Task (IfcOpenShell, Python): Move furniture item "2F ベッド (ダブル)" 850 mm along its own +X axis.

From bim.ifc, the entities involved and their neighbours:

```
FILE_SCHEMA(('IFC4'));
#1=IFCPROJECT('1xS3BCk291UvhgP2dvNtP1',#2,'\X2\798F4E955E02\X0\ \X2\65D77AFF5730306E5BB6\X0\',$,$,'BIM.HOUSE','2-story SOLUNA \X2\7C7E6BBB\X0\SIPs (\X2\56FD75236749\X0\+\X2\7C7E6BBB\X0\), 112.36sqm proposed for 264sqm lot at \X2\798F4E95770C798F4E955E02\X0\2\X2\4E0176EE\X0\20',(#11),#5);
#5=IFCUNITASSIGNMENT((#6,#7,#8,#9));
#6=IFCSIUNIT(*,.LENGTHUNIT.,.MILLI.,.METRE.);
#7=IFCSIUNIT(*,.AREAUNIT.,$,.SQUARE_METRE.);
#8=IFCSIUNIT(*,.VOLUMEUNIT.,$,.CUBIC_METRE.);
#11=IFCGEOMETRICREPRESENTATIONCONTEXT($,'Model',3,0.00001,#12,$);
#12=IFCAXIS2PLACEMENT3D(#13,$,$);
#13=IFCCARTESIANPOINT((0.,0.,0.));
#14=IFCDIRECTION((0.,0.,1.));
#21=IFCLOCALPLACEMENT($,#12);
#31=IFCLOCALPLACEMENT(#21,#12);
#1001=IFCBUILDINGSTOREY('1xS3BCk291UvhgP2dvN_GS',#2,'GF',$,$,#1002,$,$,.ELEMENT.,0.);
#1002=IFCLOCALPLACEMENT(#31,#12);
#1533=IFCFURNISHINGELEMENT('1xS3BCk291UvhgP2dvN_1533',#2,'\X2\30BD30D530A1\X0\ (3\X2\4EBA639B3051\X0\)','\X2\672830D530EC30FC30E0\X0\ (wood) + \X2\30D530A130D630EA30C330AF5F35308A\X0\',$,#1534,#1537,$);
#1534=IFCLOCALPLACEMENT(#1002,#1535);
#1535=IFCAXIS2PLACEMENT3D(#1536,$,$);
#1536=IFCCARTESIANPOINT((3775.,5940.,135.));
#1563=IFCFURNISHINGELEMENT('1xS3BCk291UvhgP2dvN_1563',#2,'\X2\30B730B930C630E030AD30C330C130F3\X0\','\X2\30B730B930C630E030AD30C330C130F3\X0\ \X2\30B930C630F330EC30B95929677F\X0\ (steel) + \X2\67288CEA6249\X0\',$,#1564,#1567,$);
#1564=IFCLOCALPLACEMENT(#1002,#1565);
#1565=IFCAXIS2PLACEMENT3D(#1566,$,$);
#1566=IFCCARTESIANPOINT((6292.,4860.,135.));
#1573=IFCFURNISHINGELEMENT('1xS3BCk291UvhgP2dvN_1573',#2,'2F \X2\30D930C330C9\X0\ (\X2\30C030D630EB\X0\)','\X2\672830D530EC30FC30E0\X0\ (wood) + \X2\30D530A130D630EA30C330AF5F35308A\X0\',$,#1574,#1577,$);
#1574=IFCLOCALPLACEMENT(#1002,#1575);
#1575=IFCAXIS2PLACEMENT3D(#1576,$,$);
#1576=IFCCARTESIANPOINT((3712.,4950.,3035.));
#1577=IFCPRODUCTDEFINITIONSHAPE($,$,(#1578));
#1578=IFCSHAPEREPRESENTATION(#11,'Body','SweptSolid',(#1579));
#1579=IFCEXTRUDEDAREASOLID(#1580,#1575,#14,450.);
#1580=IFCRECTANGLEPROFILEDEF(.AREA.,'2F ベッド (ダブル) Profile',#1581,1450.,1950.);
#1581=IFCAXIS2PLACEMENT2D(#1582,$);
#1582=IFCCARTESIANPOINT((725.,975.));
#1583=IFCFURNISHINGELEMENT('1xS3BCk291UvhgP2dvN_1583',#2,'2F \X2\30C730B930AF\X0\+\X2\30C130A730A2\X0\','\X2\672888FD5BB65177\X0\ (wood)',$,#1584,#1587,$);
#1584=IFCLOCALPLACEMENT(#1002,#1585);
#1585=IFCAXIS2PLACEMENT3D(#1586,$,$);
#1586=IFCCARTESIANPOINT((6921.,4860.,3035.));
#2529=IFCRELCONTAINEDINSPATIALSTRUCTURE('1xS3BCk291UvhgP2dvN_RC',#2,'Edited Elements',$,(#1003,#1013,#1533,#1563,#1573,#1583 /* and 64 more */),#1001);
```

```python
import ifcopenshell
import ifcopenshell.api.geometry
import ifcopenshell.util.placement
import ifcopenshell.util.unit

model = ifcopenshell.open("bim.ifc")
unit_scale = ifcopenshell.util.unit.calculate_unit_scale(model)

item = model.by_id(1573)
matrix = ifcopenshell.util.placement.get_local_placement(item.ObjectPlacement)
matrix[:3, 3] += matrix[:3, 0] * 0.85 / unit_scale
ifcopenshell.api.geometry.edit_object_placement(model, product=item, matrix=matrix, is_si=False)

print(ifcopenshell.util.placement.get_local_placement(item.ObjectPlacement).round(3) + 0.0)

model.write("bim_v2.ifc")
```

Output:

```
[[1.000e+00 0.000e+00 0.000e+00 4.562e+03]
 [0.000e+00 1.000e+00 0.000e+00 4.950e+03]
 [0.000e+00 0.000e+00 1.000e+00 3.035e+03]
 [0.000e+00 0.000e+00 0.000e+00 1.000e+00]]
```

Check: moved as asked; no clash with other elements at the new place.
